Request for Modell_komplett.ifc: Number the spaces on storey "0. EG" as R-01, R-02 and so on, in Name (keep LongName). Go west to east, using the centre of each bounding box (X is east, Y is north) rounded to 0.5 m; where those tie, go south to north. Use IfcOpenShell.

First a look at what the model holds.

```python
import ifcopenshell
import ifcopenshell.util.element
import ifcopenshell.util.placement

model = ifcopenshell.open("Modell_komplett.ifc")
print(model.schema)
storey = next(s for s in model.by_type("IfcBuildingStorey") if s.Name == "0. EG")
spaces = [e for e in ifcopenshell.util.element.get_decomposition(storey) if e.is_a("IfcSpace")]
for e in sorted(spaces, key=lambda e: e.id()):
    origin = ifcopenshell.util.placement.get_local_placement(e.ObjectPlacement)[:3, 3]
    print(e.id(), e.Name, e.LongName, origin.round(2) + 0.0, sep=" | ")
```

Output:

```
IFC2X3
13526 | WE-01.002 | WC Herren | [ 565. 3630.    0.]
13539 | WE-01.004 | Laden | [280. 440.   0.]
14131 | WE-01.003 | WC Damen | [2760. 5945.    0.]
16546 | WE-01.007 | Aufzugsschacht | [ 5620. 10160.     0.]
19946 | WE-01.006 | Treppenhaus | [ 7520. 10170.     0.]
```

```python
import ifcopenshell
import ifcopenshell.geom
import ifcopenshell.util.element
import ifcopenshell.util.shape

model = ifcopenshell.open("Modell_komplett.ifc")
settings = ifcopenshell.geom.settings()
settings.set("use-world-coords", True)


def centre(element):
    shape = ifcopenshell.geom.create_shape(settings, element)
    return ifcopenshell.util.shape.get_bbox_centroid(shape.geometry)


storey = next(s for s in model.by_type("IfcBuildingStorey") if s.Name == "0. EG")
spaces = [e for e in ifcopenshell.util.element.get_decomposition(storey) if e.is_a("IfcSpace")]

# Insertion points can sit at a corner or the storey origin, so sort by the geometry (in metres).
centres = {e: centre(e) for e in spaces}
spaces.sort(key=lambda e: (round(centres[e][0] / 0.5), centres[e][1]))

for i, e in enumerate(spaces, start=1):
    number = f"R-{i:02d}"
    e.Name = number
    print(e.id(), number)

model.write("Modell_komplett_edited.ifc")
```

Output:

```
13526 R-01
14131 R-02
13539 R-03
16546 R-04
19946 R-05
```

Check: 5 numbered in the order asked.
